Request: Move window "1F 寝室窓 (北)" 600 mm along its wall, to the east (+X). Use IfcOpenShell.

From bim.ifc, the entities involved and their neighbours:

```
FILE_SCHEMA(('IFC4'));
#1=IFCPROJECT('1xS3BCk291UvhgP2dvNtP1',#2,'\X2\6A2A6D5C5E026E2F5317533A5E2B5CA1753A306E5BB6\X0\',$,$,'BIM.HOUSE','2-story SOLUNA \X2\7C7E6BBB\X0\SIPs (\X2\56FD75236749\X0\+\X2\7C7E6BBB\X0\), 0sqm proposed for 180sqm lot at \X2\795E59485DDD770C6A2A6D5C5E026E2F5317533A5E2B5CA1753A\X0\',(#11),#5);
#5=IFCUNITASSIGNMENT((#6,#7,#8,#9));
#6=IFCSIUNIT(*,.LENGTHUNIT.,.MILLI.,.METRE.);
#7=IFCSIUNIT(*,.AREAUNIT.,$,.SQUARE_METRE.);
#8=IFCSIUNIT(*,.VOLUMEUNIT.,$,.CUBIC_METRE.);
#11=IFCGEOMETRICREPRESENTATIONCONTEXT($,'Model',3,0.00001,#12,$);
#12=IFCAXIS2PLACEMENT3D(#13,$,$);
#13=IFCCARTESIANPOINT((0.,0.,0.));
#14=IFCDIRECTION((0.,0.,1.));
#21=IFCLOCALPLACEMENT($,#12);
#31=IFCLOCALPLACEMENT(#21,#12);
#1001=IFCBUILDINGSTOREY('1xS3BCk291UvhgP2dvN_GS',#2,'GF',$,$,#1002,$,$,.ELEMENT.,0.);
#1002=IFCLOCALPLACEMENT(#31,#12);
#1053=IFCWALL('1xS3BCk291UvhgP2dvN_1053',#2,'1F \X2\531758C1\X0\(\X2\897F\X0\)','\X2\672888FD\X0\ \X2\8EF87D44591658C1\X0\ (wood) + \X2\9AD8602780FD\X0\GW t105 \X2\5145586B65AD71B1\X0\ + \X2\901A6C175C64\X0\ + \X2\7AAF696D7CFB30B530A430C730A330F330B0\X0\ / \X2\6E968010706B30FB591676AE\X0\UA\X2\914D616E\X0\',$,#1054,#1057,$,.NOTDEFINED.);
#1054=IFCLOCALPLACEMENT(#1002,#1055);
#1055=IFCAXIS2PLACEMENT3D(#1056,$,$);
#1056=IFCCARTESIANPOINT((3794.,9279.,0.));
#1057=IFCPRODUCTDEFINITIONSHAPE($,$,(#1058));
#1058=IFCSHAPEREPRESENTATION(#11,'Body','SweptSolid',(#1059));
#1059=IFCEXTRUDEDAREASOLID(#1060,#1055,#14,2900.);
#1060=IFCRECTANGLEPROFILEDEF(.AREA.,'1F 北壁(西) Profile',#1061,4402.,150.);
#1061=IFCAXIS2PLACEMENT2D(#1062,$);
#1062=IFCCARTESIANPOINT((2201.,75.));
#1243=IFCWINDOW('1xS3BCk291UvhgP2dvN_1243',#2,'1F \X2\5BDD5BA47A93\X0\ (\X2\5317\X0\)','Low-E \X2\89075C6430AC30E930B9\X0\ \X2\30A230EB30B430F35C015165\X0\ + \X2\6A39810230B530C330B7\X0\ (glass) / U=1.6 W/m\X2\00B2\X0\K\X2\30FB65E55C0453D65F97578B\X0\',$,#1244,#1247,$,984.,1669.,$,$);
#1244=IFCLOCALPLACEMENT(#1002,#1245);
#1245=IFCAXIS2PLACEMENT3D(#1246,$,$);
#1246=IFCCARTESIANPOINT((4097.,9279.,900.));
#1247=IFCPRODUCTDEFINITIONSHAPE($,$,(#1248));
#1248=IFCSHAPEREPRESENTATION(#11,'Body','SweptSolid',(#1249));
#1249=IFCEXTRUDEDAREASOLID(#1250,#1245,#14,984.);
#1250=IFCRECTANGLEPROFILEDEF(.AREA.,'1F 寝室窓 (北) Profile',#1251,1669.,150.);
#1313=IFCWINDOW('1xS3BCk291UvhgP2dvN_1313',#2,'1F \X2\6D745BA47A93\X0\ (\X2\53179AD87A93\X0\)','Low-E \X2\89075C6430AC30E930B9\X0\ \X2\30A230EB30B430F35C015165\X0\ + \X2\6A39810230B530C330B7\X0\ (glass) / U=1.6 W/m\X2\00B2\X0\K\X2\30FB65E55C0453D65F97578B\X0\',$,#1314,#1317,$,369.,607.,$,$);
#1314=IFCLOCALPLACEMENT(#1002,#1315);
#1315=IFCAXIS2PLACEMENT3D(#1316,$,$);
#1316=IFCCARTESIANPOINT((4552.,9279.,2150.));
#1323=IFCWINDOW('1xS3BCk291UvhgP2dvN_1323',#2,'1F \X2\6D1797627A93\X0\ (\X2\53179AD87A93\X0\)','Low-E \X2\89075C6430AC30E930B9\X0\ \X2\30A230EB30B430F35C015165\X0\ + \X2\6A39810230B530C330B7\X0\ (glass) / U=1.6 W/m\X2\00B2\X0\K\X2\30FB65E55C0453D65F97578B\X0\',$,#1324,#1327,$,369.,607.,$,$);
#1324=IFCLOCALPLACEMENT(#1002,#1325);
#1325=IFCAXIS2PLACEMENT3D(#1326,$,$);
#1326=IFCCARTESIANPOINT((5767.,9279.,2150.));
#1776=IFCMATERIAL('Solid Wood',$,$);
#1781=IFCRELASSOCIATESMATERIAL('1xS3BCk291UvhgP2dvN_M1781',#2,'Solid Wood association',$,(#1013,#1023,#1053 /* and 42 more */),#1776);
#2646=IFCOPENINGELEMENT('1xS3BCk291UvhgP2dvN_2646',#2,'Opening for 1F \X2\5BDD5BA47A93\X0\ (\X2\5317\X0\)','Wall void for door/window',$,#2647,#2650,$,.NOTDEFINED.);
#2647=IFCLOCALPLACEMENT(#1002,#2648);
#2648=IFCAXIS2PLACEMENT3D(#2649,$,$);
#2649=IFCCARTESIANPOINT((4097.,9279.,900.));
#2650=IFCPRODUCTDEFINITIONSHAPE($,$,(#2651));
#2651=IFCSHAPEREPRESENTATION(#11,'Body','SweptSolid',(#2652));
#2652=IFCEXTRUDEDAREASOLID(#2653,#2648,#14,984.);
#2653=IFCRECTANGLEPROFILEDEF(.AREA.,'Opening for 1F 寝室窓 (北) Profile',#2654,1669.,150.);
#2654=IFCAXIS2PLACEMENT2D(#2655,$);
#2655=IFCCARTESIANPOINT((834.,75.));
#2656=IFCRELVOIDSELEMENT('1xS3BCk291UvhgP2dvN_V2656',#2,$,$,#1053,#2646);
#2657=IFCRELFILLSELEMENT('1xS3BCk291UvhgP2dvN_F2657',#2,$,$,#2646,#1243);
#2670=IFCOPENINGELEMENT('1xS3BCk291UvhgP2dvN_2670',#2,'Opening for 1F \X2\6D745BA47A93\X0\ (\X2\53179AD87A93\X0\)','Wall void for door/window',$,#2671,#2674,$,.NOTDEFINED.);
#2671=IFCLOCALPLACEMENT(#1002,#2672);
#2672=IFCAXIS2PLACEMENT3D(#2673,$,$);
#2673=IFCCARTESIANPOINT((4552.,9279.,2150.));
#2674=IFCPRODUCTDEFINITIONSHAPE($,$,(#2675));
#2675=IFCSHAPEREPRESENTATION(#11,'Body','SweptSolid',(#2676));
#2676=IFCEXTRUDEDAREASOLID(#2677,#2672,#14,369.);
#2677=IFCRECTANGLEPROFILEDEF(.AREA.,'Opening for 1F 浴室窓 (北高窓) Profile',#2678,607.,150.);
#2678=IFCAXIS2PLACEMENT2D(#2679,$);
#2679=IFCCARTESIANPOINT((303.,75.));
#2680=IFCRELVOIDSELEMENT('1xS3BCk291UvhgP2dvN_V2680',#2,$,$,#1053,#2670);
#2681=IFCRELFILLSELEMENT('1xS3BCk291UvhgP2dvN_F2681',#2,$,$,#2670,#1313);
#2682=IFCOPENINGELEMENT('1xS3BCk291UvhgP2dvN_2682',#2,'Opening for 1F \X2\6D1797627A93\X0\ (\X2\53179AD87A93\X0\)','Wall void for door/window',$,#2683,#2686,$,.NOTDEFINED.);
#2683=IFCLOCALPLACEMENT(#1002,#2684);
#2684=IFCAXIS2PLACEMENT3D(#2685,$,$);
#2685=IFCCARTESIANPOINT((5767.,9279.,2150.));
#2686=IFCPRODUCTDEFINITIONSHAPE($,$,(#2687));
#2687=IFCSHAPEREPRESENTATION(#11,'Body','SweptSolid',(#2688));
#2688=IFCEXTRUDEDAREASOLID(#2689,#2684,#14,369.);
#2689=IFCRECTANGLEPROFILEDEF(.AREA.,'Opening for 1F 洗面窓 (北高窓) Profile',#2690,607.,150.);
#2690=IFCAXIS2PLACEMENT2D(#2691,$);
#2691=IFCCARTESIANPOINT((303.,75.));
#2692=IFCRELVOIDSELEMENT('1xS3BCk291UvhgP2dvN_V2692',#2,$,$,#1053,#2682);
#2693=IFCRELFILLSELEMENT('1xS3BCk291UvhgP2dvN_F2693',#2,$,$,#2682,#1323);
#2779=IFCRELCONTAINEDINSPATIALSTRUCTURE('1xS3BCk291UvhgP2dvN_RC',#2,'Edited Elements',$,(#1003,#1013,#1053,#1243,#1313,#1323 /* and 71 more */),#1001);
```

```python
import ifcopenshell
import ifcopenshell.api.geometry
import ifcopenshell.util.placement

model = ifcopenshell.open("bim.ifc")

window = model.by_id(1243)
opening = window.FillsVoids[0].RelatingOpeningElement
wall = opening.VoidsElements[0].RelatingBuildingElement

wall_matrix = ifcopenshell.util.placement.get_local_placement(wall.ObjectPlacement)
shift = wall_matrix[:3, 0] * 600.0
before = ifcopenshell.util.placement.get_local_placement(window.ObjectPlacement)[:3, 3].copy()

# The window is not placed relative to its opening, so move both.
for product in (opening, window):
    matrix = ifcopenshell.util.placement.get_local_placement(product.ObjectPlacement)
    matrix[:3, 3] += shift
    ifcopenshell.api.geometry.edit_object_placement(model, product=product, matrix=matrix, is_si=False)

after = ifcopenshell.util.placement.get_local_placement(window.ObjectPlacement)[:3, 3]
print("window moved by", (after - before).round(3) + 0.0)

model.write("bim_updated.ifc")
```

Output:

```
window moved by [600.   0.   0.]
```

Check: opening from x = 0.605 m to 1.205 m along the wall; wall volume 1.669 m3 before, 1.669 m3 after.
